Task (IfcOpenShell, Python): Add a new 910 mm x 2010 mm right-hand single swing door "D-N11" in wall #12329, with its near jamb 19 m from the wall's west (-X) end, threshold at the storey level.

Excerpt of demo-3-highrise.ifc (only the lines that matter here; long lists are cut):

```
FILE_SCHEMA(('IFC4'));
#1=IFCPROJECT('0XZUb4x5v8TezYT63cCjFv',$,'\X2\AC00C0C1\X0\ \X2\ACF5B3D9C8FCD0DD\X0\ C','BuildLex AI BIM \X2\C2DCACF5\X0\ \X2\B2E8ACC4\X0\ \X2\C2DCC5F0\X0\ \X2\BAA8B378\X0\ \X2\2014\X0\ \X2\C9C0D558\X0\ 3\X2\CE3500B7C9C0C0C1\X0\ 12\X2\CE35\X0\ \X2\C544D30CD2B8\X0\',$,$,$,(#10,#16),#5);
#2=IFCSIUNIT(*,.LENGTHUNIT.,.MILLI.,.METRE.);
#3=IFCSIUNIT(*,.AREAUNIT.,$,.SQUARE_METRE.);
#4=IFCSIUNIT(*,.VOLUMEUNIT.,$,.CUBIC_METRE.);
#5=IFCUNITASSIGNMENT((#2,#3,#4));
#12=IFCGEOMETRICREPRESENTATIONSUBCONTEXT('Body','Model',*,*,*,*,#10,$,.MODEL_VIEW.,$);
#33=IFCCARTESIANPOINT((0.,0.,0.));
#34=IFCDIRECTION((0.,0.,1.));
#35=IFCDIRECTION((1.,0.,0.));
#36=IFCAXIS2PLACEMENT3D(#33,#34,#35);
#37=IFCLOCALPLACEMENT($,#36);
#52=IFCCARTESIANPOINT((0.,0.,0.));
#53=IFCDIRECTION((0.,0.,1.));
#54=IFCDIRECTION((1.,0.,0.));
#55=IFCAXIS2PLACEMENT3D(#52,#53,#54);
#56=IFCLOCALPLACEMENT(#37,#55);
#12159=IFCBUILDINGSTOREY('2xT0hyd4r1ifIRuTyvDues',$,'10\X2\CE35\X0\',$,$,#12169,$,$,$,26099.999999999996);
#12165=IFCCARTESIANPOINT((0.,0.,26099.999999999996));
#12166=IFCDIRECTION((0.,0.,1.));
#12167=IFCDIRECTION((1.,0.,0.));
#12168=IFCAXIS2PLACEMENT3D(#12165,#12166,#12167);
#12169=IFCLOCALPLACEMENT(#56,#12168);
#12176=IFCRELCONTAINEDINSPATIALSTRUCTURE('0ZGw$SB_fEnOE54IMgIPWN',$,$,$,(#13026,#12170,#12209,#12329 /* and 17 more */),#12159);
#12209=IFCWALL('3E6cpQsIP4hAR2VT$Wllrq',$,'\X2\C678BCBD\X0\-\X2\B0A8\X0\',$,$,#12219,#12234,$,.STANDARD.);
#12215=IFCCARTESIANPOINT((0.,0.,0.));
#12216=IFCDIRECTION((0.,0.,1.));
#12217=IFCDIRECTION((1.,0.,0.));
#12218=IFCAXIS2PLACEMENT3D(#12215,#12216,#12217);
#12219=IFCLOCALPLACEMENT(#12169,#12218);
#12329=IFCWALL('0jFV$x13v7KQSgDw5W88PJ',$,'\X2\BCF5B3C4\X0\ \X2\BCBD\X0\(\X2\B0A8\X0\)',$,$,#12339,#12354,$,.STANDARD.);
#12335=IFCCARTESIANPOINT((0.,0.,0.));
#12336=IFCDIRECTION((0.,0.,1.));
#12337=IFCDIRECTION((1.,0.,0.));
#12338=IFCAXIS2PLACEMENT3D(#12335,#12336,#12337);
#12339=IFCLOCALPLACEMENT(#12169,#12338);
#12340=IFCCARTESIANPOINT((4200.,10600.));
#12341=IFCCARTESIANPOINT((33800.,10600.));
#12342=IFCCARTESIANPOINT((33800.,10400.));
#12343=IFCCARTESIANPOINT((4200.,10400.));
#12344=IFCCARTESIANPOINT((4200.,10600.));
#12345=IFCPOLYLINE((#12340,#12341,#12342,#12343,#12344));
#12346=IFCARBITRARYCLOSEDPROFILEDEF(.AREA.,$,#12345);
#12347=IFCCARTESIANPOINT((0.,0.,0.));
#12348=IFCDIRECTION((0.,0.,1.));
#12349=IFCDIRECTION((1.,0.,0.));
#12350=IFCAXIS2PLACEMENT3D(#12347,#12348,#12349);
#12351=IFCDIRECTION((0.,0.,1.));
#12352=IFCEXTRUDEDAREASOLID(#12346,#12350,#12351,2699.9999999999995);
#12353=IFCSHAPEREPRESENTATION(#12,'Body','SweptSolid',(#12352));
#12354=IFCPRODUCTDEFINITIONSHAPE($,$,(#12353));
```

```python
import numpy as np
import ifcopenshell
import ifcopenshell.api.feature
import ifcopenshell.api.geometry
import ifcopenshell.api.root
import ifcopenshell.api.spatial
import ifcopenshell.geom
import ifcopenshell.util.element
import ifcopenshell.util.placement
import ifcopenshell.util.representation
import ifcopenshell.util.shape
import ifcopenshell.util.unit

model = ifcopenshell.open("demo-3-highrise.ifc")
unit_scale = ifcopenshell.util.unit.calculate_unit_scale(model)
settings = ifcopenshell.geom.settings()


def volume(element):
    """Net volume in cubic metres, openings subtracted."""
    shape = ifcopenshell.geom.create_shape(settings, element)
    return ifcopenshell.util.shape.get_volume(shape.geometry)


wall = model.by_guid("0jFV$x13v7KQSgDw5W88PJ")
storey = ifcopenshell.util.element.get_container(wall, ifc_class="IfcBuildingStorey")
context = ifcopenshell.util.representation.get_context(model, "Model", "Body", "MODEL_VIEW")
before = volume(wall)

width, height, from_end, sill = 0.91, 2.01, 19, 0.0  # metres

# The wall runs along its own X axis, and the end named is its -X end.
wall_shape = ifcopenshell.geom.create_shape(settings, wall)
x, y, z = ifcopenshell.util.shape.get_vertices(wall_shape.geometry).T
start = x.min() + from_end
face, thickness = float(y.min()), float(y.max() - y.min())
wall_matrix = ifcopenshell.util.placement.get_local_placement(wall.ObjectPlacement)
level = ifcopenshell.util.placement.get_local_placement(storey.ObjectPlacement)[2, 3]


def in_wall(x, y):
    """Placement at x, y metres in the wall's axes, at sill height."""
    matrix = wall_matrix.copy()
    matrix[:, 3] = wall_matrix @ np.array([x / unit_scale, y / unit_scale, 0.0, 1.0])
    matrix[2, 3] = level + sill / unit_scale
    return matrix


# Opening: a box that overshoots both wall faces by 50 mm.
opening = ifcopenshell.api.root.create_entity(model, ifc_class="IfcOpeningElement", predefined_type="OPENING")
box = ifcopenshell.api.geometry.add_wall_representation(
    model, context=context, length=width, height=height, thickness=thickness + 0.1
)
ifcopenshell.api.geometry.assign_representation(model, product=opening, representation=box)
ifcopenshell.api.geometry.edit_object_placement(model, product=opening, matrix=in_wall(start, face - 0.05), is_si=False)
ifcopenshell.api.feature.add_feature(model, feature=opening, element=wall)

door = ifcopenshell.api.root.create_entity(model, ifc_class="IfcDoor", name="D-N11", predefined_type="DOOR")
door.OverallWidth, door.OverallHeight = width / unit_scale, height / unit_scale
door.OperationType = "SINGLE_SWING_RIGHT"
body = ifcopenshell.api.geometry.add_door_representation(
    model,
    context=context,
    overall_width=door.OverallWidth,
    overall_height=door.OverallHeight,
    operation_type="SINGLE_SWING_RIGHT",
    lining_properties={"LiningDepth": thickness / unit_scale, "ThresholdDepth": thickness / unit_scale},
)
ifcopenshell.api.geometry.assign_representation(model, product=door, representation=body)
ifcopenshell.api.spatial.assign_container(model, products=[door], relating_structure=storey)
ifcopenshell.api.feature.add_filling(model, opening=opening, element=door)

# The lining spans the wall, so the door starts at the wall face.
ifcopenshell.api.geometry.edit_object_placement(model, product=door, matrix=in_wall(start, face), is_si=False)

after = volume(wall)

print(f"wall volume {before:.3f} -> {after:.3f} m3")

model.write("demo-3-highrise_v2.ifc")
```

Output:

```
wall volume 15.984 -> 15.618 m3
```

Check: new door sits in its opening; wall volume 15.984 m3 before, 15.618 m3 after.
